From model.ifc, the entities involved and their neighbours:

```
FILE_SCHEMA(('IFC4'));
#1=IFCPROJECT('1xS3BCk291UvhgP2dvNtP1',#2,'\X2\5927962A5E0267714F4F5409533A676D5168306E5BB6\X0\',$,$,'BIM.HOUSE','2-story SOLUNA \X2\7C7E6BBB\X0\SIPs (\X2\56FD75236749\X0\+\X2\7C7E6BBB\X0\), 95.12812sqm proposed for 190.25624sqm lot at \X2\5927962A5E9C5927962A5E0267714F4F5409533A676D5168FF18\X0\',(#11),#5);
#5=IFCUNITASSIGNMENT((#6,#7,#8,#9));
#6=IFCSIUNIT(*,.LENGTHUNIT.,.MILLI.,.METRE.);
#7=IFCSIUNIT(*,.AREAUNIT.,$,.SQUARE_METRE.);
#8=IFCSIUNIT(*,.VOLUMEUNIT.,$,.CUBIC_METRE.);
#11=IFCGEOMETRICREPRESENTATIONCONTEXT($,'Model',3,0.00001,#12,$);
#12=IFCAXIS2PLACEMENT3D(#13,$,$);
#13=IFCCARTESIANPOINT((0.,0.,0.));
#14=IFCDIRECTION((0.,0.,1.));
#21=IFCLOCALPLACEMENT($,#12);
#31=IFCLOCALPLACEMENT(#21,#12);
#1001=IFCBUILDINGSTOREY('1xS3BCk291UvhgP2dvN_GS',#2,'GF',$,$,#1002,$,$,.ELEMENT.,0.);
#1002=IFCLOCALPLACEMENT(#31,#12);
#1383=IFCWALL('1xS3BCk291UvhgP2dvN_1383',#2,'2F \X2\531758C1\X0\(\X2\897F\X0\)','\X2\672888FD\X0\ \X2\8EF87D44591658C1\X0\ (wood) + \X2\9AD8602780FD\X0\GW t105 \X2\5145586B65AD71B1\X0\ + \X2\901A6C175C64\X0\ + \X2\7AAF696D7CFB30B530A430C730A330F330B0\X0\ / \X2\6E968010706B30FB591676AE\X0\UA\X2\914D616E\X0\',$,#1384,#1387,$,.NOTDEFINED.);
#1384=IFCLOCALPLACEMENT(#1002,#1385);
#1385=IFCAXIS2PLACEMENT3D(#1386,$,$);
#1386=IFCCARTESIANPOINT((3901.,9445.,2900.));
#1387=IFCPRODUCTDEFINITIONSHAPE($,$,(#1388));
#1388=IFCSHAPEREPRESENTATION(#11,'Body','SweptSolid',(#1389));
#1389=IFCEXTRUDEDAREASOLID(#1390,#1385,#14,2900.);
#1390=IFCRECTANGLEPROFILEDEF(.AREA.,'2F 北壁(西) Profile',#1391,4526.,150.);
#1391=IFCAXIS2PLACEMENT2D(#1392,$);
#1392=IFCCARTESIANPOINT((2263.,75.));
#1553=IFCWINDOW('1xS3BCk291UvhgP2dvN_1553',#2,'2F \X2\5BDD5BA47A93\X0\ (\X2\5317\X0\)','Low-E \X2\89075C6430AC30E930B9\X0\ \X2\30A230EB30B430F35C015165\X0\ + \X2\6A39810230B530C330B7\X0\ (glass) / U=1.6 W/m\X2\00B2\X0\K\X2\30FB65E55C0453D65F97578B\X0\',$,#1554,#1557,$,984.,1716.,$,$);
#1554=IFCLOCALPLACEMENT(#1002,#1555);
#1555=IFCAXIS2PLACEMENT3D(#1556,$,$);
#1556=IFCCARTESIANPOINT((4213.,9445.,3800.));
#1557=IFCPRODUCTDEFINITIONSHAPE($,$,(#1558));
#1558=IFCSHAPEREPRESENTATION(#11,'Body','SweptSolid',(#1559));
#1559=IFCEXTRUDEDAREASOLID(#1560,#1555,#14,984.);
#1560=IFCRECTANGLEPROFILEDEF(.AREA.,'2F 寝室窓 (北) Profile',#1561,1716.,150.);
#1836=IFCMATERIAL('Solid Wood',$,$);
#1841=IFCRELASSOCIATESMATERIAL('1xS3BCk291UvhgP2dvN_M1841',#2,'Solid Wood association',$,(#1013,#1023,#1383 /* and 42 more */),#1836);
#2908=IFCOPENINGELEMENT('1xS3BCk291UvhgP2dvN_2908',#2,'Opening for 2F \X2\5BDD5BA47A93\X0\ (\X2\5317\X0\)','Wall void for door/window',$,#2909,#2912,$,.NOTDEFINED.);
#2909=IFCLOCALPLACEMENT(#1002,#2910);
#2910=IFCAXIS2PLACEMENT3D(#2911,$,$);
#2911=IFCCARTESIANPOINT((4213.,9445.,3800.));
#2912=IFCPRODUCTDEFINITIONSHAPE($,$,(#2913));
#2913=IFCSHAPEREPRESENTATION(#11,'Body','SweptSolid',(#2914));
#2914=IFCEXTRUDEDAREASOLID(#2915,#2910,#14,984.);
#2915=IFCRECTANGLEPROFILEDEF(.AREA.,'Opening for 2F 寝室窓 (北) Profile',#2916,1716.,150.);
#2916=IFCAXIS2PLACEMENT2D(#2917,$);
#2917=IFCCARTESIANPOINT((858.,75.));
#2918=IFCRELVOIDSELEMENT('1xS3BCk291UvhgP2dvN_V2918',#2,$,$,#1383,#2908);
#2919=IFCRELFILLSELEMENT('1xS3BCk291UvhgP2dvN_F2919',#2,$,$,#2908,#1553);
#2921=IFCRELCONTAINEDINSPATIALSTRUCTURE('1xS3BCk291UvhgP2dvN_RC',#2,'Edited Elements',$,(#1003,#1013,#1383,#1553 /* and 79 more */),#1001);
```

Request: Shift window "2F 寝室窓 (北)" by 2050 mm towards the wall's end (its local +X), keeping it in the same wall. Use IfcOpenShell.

```python
import ifcopenshell
import ifcopenshell.api.geometry
import ifcopenshell.util.placement

model = ifcopenshell.open("model.ifc")

window = model.by_id(1553)
opening = window.FillsVoids[0].RelatingOpeningElement
wall = opening.VoidsElements[0].RelatingBuildingElement

wall_matrix = ifcopenshell.util.placement.get_local_placement(wall.ObjectPlacement)
shift = wall_matrix[:3, 0] * 2050.0
before = ifcopenshell.util.placement.get_local_placement(window.ObjectPlacement)[:3, 3].copy()

# The window is not placed relative to its opening, so move both.
for product in (opening, window):
    matrix = ifcopenshell.util.placement.get_local_placement(product.ObjectPlacement)
    matrix[:3, 3] += shift
    ifcopenshell.api.geometry.edit_object_placement(model, product=product, matrix=matrix, is_si=False)

after = ifcopenshell.util.placement.get_local_placement(window.ObjectPlacement)[:3, 3]
print("window moved by", (after - before).round(3) + 0.0)

model.write("model_updated.ifc")
```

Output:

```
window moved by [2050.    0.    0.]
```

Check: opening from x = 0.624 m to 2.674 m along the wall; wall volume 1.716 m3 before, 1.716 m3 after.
